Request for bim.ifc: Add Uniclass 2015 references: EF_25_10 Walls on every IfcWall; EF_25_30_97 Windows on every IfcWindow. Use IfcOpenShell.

First a look at what the model holds.

```python
import ifcopenshell

model = ifcopenshell.open("bim.ifc")
print(model.schema)
print("classifications:", [c.Name for c in model.by_type("IfcClassification")])
for ifc_class in ("IfcDoor", "IfcRoof", "IfcStair", "IfcWall", "IfcWindow"):
    print(ifc_class, len(model.by_type(ifc_class)))
```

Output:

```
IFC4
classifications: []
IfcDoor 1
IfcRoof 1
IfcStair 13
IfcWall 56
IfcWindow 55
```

```python
import ifcopenshell
import ifcopenshell.api.classification

model = ifcopenshell.open("bim.ifc")

system = ifcopenshell.api.classification.add_classification(model, classification="Uniclass 2015")

codes = {
    "IfcWall": ("EF_25_10", "Walls"),
    "IfcWindow": ("EF_25_30_97", "Windows"),
}
for ifc_class, (code, name) in codes.items():
    products = model.by_type(ifc_class)
    ifcopenshell.api.classification.add_reference(
        model, products=products, classification=system, identification=code, name=name
    )
    print(code, len(products))

model.write("bim_v2.ifc")
```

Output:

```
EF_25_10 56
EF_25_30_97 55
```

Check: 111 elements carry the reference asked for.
